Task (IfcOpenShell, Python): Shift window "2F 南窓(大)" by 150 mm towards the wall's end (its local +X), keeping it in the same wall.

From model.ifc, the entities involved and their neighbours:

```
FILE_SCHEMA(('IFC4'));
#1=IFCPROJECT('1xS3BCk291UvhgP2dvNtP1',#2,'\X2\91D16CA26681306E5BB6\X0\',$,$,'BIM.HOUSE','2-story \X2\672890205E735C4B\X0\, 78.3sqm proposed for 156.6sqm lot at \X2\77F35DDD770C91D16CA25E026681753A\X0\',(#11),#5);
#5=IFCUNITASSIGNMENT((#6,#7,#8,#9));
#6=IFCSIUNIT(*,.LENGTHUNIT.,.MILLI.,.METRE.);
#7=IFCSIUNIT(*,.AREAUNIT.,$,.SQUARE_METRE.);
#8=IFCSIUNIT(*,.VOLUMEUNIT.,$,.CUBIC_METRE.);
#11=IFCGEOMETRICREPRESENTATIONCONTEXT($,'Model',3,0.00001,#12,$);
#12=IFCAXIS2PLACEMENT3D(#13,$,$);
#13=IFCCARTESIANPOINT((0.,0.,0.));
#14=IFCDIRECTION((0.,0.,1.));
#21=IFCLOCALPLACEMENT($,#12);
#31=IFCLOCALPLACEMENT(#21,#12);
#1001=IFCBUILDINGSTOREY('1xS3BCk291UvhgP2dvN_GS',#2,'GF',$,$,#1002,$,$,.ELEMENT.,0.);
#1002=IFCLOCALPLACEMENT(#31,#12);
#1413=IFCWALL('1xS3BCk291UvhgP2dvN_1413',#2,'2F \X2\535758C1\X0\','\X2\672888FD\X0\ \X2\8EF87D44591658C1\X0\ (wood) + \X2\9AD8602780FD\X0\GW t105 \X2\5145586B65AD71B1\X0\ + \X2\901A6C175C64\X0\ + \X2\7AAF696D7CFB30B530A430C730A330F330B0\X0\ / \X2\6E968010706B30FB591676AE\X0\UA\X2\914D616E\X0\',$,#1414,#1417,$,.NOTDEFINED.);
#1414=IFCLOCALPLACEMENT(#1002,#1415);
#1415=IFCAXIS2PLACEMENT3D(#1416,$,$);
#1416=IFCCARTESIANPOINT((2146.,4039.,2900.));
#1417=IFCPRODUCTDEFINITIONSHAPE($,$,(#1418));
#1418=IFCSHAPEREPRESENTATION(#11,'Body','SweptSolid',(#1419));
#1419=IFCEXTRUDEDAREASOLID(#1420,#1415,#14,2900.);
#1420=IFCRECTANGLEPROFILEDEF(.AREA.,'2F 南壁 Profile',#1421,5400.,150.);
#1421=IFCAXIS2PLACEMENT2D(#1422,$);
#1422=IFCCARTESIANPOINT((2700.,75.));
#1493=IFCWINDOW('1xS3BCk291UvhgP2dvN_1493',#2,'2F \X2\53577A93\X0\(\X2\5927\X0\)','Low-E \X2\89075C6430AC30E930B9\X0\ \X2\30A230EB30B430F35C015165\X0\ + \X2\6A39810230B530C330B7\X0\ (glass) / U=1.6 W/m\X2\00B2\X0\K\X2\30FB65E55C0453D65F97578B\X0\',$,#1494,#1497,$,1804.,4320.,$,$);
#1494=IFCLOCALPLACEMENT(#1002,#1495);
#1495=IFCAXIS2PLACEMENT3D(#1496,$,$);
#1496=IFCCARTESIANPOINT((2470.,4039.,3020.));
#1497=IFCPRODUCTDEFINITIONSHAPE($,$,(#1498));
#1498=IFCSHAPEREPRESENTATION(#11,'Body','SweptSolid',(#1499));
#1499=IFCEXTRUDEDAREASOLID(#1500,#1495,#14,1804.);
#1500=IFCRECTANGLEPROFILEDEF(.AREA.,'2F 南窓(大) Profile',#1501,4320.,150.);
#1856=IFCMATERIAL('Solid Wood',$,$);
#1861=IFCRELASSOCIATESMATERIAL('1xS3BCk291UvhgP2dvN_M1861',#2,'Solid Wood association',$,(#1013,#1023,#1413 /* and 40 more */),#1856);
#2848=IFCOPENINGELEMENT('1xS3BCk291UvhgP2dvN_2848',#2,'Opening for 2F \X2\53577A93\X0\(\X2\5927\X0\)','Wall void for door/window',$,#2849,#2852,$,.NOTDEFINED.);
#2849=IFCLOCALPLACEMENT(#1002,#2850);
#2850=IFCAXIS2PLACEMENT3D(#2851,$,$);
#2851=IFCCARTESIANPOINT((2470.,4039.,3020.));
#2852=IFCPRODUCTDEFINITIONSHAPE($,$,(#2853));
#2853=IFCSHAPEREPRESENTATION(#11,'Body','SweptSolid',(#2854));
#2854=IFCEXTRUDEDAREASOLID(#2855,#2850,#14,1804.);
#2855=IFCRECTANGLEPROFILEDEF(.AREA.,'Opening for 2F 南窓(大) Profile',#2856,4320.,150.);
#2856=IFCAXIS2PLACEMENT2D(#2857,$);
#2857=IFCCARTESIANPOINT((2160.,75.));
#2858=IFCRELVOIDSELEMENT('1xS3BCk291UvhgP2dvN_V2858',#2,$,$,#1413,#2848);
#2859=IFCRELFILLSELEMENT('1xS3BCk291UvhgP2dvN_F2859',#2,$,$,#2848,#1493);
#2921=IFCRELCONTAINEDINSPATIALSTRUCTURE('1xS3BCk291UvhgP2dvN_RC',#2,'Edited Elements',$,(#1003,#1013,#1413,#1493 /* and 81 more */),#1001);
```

```python
import ifcopenshell
import ifcopenshell.api.geometry
import ifcopenshell.util.placement
import ifcopenshell.util.unit

model = ifcopenshell.open("model.ifc")
unit_scale = ifcopenshell.util.unit.calculate_unit_scale(model)

window = model.by_guid("1xS3BCk291UvhgP2dvN_1493")
opening = window.FillsVoids[0].RelatingOpeningElement
wall = opening.VoidsElements[0].RelatingBuildingElement

wall_matrix = ifcopenshell.util.placement.get_local_placement(wall.ObjectPlacement)
shift = wall_matrix[:3, 0] * 0.15 / unit_scale
before = ifcopenshell.util.placement.get_local_placement(window.ObjectPlacement)[:3, 3].copy()

# The window is not placed relative to its opening, so move both.
for product in (opening, window):
    matrix = ifcopenshell.util.placement.get_local_placement(product.ObjectPlacement)
    matrix[:3, 3] += shift
    ifcopenshell.api.geometry.edit_object_placement(model, product=product, matrix=matrix, is_si=False)

after = ifcopenshell.util.placement.get_local_placement(window.ObjectPlacement)[:3, 3]
print("window moved by", (after - before).round(3) + 0.0)

model.write("model_v2.ifc")
```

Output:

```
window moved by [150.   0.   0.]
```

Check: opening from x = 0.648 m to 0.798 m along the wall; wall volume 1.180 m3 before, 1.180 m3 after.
